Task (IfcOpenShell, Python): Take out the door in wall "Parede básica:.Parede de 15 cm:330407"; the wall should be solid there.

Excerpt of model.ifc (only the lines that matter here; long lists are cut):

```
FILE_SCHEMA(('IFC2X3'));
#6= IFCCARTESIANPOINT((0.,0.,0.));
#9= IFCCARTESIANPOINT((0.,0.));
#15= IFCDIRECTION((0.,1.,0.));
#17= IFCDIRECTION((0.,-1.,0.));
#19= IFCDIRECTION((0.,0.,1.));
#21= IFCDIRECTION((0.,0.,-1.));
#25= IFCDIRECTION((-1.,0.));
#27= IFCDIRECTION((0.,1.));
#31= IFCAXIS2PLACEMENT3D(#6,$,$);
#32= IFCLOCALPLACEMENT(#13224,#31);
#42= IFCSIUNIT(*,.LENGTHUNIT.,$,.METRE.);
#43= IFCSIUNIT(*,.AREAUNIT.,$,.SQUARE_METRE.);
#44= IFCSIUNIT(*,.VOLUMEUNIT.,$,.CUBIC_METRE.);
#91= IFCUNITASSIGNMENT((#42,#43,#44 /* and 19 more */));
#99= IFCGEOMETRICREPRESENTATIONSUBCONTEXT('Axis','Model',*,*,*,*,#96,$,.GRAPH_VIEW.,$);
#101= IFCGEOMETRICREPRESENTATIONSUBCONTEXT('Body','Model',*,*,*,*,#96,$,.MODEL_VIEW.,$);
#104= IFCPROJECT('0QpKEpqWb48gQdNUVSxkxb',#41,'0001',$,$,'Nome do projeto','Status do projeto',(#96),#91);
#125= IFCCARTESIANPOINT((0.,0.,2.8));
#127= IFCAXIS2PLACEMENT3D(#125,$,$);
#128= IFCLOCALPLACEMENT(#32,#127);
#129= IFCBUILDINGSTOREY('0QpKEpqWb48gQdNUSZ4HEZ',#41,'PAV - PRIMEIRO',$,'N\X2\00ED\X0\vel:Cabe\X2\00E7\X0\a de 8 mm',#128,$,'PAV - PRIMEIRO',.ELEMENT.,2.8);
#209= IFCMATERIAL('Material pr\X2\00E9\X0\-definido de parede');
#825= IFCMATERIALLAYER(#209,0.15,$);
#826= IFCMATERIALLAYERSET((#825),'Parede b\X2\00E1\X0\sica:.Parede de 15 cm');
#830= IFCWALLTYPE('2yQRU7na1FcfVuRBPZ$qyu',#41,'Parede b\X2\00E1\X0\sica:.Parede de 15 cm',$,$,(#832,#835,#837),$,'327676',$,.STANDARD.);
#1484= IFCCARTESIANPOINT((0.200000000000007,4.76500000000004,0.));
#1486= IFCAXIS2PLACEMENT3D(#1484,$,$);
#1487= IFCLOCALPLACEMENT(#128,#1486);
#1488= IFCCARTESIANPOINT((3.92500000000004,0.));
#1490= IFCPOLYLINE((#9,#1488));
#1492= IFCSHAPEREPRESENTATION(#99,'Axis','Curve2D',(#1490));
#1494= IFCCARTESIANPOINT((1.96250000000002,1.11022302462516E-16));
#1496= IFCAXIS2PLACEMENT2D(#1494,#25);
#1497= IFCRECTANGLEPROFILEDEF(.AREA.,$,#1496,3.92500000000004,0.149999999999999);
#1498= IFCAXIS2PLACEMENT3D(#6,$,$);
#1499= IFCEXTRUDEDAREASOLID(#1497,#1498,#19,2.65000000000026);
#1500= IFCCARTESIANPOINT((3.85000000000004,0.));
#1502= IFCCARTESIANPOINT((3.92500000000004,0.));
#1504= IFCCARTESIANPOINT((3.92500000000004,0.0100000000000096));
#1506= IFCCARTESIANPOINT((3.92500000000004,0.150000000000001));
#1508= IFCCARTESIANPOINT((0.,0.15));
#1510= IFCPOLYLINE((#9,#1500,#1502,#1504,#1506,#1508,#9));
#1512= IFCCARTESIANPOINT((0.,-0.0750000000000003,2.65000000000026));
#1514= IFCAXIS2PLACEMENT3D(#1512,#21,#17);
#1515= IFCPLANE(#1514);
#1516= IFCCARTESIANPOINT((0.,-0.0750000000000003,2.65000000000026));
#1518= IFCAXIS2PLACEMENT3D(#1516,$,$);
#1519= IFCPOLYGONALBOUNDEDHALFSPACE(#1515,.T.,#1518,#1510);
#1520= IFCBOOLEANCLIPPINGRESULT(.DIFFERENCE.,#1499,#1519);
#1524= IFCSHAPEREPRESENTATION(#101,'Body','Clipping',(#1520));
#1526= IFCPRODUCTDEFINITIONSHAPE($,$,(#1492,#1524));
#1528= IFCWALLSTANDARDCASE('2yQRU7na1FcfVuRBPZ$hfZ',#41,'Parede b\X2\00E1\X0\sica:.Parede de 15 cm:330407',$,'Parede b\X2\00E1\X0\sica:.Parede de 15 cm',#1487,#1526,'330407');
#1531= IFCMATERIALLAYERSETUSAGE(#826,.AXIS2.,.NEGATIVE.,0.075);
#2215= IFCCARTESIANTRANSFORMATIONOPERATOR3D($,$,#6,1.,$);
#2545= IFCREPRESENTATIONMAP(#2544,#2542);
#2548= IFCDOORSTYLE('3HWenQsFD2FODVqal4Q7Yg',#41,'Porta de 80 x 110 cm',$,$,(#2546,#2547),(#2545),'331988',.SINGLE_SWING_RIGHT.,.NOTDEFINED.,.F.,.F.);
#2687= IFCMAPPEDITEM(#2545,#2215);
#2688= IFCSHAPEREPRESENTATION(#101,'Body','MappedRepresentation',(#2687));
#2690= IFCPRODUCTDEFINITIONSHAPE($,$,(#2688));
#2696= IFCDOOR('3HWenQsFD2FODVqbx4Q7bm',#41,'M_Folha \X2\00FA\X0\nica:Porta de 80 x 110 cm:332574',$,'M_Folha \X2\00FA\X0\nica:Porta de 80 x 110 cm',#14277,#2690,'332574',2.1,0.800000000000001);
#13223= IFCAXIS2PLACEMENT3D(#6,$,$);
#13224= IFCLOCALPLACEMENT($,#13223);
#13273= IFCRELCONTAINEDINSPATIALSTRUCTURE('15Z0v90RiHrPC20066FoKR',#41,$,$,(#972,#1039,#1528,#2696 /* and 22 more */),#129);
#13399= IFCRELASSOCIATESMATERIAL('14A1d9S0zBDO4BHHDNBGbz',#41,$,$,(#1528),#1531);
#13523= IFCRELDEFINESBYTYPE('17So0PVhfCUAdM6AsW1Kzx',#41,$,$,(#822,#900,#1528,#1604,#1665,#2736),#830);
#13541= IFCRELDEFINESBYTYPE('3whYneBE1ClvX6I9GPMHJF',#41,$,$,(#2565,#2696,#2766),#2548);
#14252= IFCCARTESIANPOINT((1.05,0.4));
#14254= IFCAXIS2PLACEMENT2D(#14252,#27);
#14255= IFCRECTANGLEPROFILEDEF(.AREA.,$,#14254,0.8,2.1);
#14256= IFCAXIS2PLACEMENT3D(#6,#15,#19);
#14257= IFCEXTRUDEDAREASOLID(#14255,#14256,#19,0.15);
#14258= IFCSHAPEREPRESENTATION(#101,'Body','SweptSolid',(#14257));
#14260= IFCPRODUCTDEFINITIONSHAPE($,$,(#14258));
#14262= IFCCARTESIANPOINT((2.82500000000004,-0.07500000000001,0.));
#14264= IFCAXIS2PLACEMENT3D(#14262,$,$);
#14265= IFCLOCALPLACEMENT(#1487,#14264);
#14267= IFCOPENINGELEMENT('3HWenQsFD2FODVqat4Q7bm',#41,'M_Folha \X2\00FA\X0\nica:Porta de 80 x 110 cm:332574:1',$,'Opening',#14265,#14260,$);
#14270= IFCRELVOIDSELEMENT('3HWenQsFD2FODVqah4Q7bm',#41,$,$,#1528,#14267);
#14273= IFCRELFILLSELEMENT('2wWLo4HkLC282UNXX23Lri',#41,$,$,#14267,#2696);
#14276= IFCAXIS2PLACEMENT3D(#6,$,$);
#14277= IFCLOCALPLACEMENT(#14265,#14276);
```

```python
import ifcopenshell
import ifcopenshell.api.feature
import ifcopenshell.api.root
import ifcopenshell.geom
import ifcopenshell.util.shape

model = ifcopenshell.open("model.ifc")
settings = ifcopenshell.geom.settings()


def volume(element):
    """Net volume in cubic metres, openings subtracted."""
    shape = ifcopenshell.geom.create_shape(settings, element)
    return ifcopenshell.util.shape.get_volume(shape.geometry)


door = model.by_id(2696)
opening = door.FillsVoids[0].RelatingOpeningElement
wall = opening.VoidsElements[0].RelatingBuildingElement
before = volume(wall)

ifcopenshell.api.root.remove_product(model, product=door)
ifcopenshell.api.feature.remove_feature(model, feature=opening)

after = volume(wall)

print(f"wall volume {before:.3f} -> {after:.3f} m3")

model.write("model_v2.ifc")
```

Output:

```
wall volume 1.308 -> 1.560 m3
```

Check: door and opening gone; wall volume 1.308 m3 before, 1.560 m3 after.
